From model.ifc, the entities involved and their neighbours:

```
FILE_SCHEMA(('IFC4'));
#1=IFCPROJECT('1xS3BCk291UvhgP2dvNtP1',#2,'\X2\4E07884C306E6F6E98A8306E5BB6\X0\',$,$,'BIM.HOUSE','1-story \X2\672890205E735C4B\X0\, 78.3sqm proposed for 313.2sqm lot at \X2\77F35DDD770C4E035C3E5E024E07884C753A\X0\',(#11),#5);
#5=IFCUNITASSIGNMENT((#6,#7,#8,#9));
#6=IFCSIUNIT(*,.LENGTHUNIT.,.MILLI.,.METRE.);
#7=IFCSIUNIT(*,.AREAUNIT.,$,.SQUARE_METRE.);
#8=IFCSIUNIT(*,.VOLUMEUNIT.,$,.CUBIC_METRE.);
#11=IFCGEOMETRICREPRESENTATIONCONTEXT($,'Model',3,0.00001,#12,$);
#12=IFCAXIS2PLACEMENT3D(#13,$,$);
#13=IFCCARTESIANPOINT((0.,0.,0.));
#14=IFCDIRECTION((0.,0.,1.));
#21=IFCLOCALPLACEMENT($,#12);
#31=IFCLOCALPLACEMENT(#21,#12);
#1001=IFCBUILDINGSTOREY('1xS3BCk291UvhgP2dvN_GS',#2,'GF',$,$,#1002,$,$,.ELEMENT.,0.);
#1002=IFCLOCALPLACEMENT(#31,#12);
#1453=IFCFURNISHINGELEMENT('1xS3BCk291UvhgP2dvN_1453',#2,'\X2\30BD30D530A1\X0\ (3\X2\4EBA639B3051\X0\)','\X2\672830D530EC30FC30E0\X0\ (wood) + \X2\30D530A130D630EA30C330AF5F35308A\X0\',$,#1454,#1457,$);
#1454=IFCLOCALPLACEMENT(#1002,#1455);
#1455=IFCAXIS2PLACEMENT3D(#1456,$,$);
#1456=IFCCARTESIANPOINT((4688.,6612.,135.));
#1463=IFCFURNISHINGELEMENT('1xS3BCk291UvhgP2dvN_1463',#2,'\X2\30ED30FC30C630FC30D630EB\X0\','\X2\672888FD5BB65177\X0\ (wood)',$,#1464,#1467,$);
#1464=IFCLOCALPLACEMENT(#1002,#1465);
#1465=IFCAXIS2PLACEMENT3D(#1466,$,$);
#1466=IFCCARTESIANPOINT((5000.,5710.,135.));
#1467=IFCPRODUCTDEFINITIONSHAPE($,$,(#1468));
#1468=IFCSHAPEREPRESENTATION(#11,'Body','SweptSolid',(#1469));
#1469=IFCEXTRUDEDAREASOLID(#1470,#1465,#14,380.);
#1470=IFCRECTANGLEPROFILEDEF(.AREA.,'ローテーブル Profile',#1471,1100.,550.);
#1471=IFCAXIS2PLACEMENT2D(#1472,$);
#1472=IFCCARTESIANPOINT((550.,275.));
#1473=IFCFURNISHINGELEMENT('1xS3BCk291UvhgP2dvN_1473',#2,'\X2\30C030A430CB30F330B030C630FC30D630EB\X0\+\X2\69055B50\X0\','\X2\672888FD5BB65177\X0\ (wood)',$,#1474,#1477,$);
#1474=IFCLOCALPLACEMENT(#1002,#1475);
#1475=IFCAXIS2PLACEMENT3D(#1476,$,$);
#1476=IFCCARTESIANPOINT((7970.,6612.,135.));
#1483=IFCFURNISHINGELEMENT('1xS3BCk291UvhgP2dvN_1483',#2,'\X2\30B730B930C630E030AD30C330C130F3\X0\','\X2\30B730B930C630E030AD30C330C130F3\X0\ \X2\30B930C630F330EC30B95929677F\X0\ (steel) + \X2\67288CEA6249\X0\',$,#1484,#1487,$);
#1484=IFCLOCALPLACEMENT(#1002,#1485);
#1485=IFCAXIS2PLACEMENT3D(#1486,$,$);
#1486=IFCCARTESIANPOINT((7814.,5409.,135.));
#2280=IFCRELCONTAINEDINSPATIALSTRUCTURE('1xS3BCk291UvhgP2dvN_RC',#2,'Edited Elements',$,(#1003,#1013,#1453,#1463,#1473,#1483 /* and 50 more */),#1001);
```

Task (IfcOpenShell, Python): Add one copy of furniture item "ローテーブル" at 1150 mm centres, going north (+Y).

```python
import numpy as np
import ifcopenshell
import ifcopenshell.api.geometry
import ifcopenshell.api.root
import ifcopenshell.util.element
import ifcopenshell.util.placement
import ifcopenshell.util.unit

model = ifcopenshell.open("model.ifc")
unit_scale = ifcopenshell.util.unit.calculate_unit_scale(model)


def reuse_history(source, copy):
    """copy_class also copies each property set's owner history, people and application; keep the originals."""
    for rel in copy.IsDefinedBy:
        if rel.is_a("IfcRelDefinesByProperties") and (history := rel.RelatingPropertyDefinition.OwnerHistory):
            rel.RelatingPropertyDefinition.OwnerHistory = source.OwnerHistory
            ifcopenshell.util.element.remove_deep2(model, history)


source = model.by_guid("1xS3BCk291UvhgP2dvN_1463")
base = ifcopenshell.util.placement.get_local_placement(source.ObjectPlacement)
step = np.array([0.0, 1.0, 0.0]) * 1.15 / unit_scale

for i in range(1, 2):
    copy = ifcopenshell.api.root.copy_class(model, product=source)
    copy.Representation = ifcopenshell.util.element.copy_deep(
        model, source.Representation, exclude=["IfcGeometricRepresentationContext", "IfcRepresentationMap"]
    )
    reuse_history(source, copy)
    matrix = base.copy()
    matrix[:3, 3] += i * step
    print("added at", matrix[:3, 3].round(3) + 0.0)
    ifcopenshell.api.geometry.edit_object_placement(model, product=copy, matrix=matrix, is_si=False)

model.write("model_edited.ifc")
```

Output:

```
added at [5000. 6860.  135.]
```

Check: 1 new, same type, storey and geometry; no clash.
